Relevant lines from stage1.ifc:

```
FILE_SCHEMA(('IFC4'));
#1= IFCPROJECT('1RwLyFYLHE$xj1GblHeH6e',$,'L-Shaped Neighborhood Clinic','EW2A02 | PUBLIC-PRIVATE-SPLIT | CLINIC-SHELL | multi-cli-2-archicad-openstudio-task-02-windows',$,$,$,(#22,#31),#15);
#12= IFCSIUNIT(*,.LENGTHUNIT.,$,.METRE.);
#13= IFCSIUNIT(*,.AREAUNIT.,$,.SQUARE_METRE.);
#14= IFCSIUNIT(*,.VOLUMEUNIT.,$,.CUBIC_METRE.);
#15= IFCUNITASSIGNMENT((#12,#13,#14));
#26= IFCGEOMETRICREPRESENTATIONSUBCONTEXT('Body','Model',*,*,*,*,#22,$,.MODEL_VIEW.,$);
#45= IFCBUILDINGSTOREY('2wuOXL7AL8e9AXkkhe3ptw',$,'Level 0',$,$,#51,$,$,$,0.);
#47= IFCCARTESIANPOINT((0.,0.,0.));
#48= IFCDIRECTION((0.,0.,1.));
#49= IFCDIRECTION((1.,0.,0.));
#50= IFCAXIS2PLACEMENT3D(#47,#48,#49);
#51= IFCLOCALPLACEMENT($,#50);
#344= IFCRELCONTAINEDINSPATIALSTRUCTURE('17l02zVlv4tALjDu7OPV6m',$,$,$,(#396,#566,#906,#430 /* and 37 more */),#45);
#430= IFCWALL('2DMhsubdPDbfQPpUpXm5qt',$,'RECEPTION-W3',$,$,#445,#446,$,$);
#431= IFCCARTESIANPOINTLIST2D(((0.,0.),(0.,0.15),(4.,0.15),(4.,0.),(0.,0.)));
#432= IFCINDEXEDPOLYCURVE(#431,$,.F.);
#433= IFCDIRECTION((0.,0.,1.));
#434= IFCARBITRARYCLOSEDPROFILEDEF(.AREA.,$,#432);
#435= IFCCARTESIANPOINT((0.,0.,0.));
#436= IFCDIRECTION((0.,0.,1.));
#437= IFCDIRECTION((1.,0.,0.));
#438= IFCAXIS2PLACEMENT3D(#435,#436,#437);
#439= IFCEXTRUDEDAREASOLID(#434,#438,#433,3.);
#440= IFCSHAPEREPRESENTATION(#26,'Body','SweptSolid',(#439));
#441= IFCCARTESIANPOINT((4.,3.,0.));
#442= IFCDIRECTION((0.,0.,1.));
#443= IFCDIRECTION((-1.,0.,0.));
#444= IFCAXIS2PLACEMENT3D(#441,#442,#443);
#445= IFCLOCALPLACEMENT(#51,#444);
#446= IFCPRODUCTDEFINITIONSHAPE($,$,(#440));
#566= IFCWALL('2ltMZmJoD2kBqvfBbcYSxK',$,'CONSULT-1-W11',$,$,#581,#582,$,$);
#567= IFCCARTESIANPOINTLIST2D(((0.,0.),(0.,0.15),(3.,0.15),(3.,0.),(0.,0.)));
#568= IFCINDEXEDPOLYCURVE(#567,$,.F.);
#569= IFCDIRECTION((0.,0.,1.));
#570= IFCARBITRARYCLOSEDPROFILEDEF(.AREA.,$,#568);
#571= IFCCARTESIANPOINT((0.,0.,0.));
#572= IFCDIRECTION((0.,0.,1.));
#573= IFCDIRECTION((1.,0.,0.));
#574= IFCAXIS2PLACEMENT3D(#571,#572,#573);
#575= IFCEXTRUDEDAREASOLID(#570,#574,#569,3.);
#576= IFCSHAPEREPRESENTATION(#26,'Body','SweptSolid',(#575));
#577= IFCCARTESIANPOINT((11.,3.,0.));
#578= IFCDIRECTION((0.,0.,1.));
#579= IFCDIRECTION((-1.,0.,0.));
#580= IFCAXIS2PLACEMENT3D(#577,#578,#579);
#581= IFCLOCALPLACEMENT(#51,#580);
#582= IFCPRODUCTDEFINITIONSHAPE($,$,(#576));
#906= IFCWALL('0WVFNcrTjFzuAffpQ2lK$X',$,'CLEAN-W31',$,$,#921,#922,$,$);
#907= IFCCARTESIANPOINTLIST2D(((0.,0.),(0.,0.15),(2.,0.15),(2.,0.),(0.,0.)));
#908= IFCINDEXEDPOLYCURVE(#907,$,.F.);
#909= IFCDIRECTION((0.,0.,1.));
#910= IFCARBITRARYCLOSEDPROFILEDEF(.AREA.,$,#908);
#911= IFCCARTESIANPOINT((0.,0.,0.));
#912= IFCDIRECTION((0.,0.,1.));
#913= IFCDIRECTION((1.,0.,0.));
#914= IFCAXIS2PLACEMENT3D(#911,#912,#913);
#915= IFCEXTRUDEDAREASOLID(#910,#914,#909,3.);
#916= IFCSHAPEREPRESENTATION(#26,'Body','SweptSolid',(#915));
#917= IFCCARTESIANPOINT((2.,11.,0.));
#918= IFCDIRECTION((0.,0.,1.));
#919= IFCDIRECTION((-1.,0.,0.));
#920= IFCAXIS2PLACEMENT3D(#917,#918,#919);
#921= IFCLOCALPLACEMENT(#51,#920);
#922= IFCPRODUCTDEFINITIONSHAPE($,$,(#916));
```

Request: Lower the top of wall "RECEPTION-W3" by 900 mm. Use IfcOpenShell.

```python
import ifcopenshell
import ifcopenshell.geom
import ifcopenshell.util.representation
import ifcopenshell.util.shape

model = ifcopenshell.open("stage1.ifc")
settings = ifcopenshell.geom.settings()


def volume(element):
    """Net volume in cubic metres, openings subtracted."""
    shape = ifcopenshell.geom.create_shape(settings, element)
    return ifcopenshell.util.shape.get_volume(shape.geometry)


wall = model.by_guid("2DMhsubdPDbfQPpUpXm5qt")
before = volume(wall)

body = ifcopenshell.util.representation.get_representation(wall, "Model", "Body")
solid = body.Items[0]
old_height = solid.Depth
solid.Depth -= 0.9
after = volume(wall)

print(f"height {old_height:g} -> {solid.Depth:g}, volume {before:.3f} -> {after:.3f} m3")

model.write("stage1_v2.ifc")
```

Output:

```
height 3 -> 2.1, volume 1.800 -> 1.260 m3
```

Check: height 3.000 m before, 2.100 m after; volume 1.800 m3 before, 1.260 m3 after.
